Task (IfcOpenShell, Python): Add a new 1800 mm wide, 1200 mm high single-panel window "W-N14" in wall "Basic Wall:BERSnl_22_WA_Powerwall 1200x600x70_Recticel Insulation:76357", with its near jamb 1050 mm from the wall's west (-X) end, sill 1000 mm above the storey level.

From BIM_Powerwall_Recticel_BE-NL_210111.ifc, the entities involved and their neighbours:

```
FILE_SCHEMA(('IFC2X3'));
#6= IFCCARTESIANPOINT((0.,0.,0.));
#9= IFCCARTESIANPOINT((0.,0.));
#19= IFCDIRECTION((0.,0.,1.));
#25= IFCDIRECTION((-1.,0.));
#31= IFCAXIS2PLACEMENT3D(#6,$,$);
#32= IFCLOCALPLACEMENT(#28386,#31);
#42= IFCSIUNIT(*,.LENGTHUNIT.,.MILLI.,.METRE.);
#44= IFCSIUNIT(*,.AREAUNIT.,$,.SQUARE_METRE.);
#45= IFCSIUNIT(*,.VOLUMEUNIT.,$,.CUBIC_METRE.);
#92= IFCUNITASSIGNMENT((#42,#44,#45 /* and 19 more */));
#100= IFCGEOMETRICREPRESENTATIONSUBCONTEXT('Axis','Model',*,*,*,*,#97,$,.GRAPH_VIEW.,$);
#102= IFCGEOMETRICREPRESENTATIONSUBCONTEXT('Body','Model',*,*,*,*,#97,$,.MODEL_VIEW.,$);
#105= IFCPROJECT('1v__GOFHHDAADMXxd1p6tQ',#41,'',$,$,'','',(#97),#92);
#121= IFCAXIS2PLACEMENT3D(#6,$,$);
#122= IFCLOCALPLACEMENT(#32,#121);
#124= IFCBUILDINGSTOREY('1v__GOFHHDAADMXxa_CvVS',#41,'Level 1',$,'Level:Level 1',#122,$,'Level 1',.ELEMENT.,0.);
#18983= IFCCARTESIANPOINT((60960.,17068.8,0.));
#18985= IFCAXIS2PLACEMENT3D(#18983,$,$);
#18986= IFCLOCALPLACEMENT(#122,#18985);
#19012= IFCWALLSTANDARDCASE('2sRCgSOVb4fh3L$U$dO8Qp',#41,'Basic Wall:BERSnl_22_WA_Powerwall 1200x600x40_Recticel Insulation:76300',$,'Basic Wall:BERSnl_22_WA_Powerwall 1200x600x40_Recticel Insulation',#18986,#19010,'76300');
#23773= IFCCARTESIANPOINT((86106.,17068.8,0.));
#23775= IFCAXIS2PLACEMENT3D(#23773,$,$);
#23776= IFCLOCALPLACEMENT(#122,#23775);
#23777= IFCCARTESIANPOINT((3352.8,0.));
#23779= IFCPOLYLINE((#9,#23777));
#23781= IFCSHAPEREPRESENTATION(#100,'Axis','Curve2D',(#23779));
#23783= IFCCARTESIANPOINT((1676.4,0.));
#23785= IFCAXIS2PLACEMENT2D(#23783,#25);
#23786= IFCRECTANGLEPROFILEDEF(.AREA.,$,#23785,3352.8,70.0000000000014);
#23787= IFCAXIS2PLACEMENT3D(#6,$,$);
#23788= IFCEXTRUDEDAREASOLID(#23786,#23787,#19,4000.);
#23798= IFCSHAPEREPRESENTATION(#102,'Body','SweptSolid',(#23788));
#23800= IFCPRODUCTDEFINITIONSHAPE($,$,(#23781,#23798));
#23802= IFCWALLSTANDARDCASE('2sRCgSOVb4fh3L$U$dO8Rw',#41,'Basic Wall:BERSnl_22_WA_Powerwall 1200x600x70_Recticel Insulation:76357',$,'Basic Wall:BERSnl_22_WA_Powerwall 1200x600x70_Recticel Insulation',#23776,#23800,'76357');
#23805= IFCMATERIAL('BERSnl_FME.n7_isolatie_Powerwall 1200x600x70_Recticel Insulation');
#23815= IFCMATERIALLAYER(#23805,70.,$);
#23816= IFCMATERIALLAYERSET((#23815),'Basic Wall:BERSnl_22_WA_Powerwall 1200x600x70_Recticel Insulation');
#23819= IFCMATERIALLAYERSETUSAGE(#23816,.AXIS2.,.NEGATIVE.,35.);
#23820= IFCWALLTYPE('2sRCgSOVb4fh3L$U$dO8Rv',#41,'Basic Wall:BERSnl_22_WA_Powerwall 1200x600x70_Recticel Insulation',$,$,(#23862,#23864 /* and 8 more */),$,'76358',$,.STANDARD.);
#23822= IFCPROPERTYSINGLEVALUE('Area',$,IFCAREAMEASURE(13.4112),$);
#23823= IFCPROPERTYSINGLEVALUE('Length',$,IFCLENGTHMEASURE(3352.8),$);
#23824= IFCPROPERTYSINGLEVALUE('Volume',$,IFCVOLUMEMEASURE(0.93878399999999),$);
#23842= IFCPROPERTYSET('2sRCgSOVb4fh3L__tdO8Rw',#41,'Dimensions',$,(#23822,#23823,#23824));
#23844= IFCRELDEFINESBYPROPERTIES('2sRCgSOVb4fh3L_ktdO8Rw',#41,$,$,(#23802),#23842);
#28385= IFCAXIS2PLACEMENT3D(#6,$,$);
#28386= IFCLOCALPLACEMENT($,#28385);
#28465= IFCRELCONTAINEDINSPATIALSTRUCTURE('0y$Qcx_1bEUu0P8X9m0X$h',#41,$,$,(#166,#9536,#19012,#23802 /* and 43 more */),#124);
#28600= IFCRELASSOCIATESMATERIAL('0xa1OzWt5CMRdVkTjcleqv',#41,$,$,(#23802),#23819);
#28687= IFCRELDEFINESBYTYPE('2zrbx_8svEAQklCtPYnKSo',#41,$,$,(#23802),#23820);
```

```python
import numpy as np
import ifcopenshell
import ifcopenshell.api.feature
import ifcopenshell.api.geometry
import ifcopenshell.api.pset
import ifcopenshell.api.root
import ifcopenshell.api.spatial
import ifcopenshell.api.type
import ifcopenshell.geom
import ifcopenshell.util.element
import ifcopenshell.util.placement
import ifcopenshell.util.representation
import ifcopenshell.util.shape
import ifcopenshell.util.unit

model = ifcopenshell.open("BIM_Powerwall_Recticel_BE-NL_210111.ifc")
unit_scale = ifcopenshell.util.unit.calculate_unit_scale(model)
area_scale = ifcopenshell.util.unit.calculate_unit_scale(model, "AREAUNIT")
volume_scale = ifcopenshell.util.unit.calculate_unit_scale(model, "VOLUMEUNIT")
settings = ifcopenshell.geom.settings()


def volume(element):
    """Net volume in cubic metres, openings subtracted."""
    shape = ifcopenshell.geom.create_shape(settings, element)
    return ifcopenshell.util.shape.get_volume(shape.geometry)


wall = model.by_id(23802)
storey = ifcopenshell.util.element.get_container(wall, ifc_class="IfcBuildingStorey")
context = ifcopenshell.util.representation.get_context(model, "Model", "Body", "MODEL_VIEW")
before = volume(wall)

width, height, from_end, sill = 1.8, 1.2, 1.05, 1  # metres

# The wall runs along its own X axis, and the end named is its -X end.
wall_shape = ifcopenshell.geom.create_shape(settings, wall)
x, y, z = ifcopenshell.util.shape.get_vertices(wall_shape.geometry).T
start = x.min() + from_end
face, thickness = float(y.min()), float(y.max() - y.min())
wall_matrix = ifcopenshell.util.placement.get_local_placement(wall.ObjectPlacement)
level = ifcopenshell.util.placement.get_local_placement(storey.ObjectPlacement)[2, 3]


def in_wall(x, y):
    """Placement at x, y metres in the wall's axes, at sill height."""
    matrix = wall_matrix.copy()
    matrix[:, 3] = wall_matrix @ np.array([x / unit_scale, y / unit_scale, 0.0, 1.0])
    matrix[2, 3] = level + sill / unit_scale
    return matrix


# Opening: a box that overshoots both wall faces by 50 mm.
opening = ifcopenshell.api.root.create_entity(model, ifc_class="IfcOpeningElement")
box = ifcopenshell.api.geometry.add_wall_representation(
    model, context=context, length=width, height=height, thickness=thickness + 0.1
)
ifcopenshell.api.geometry.assign_representation(model, product=opening, representation=box)
ifcopenshell.api.geometry.edit_object_placement(model, product=opening, matrix=in_wall(start, face - 0.05), is_si=False)
ifcopenshell.api.feature.add_feature(model, feature=opening, element=wall)

window = ifcopenshell.api.root.create_entity(model, ifc_class="IfcWindow", name="W-N14")
window.OverallWidth, window.OverallHeight = width / unit_scale, height / unit_scale
body = ifcopenshell.api.geometry.add_window_representation(
    model,
    context=context,
    overall_width=window.OverallWidth,
    overall_height=window.OverallHeight,
    partition_type="SINGLE_PANEL",
)
ifcopenshell.api.geometry.assign_representation(model, product=window, representation=body)
ifcopenshell.api.spatial.assign_container(model, products=[window], relating_structure=storey)
fills = ifcopenshell.api.feature.add_filling(model, opening=opening, element=window)
fills.OwnerHistory = window.OwnerHistory  # required in IFC2X3

# IFC2X3 keeps the operation on the window style.
style = ifcopenshell.api.root.create_entity(model, ifc_class="IfcWindowStyle", name="W-N14")
style.OperationType, style.ConstructionType = "SINGLE_PANEL", "NOTDEFINED"
style.ParameterTakesPrecedence = style.Sizeable = False
ifcopenshell.api.type.assign_type(model, related_objects=[window], relating_type=style)

# Centre the window in the wall's thickness.
ifcopenshell.api.geometry.edit_object_placement(model, product=window, matrix=in_wall(start, face), is_si=False)
window_shape = ifcopenshell.geom.create_shape(settings, window)
depth = ifcopenshell.util.shape.get_vertices(window_shape.geometry)[:, 1]
offset = face + thickness / 2 - (depth.min() + depth.max()) / 2
ifcopenshell.api.geometry.edit_object_placement(model, product=window, matrix=in_wall(start, offset), is_si=False)

after = volume(wall)

# Update the wall's stored quantities.
pset = model.by_id(ifcopenshell.util.element.get_pset(wall, "Dimensions", should_inherit=False)["id"])
ifcopenshell.api.pset.edit_pset(model, pset=pset, properties={
    "Area": model.create_entity("IfcAreaMeasure", after / thickness / area_scale),
    "Volume": model.create_entity("IfcVolumeMeasure", after / volume_scale),
})

print(f"wall volume {before:.3f} -> {after:.3f} m3")

model.write("BIM_Powerwall_Recticel_BE-NL_210111_rev.ifc")
```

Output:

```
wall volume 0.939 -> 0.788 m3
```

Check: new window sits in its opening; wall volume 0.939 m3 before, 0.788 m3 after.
